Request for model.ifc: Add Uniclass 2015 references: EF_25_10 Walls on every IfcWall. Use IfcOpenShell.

First a look at what the model holds.

```python
import ifcopenshell

model = ifcopenshell.open("model.ifc")
print(model.schema)
print("classifications:", [c.Name for c in model.by_type("IfcClassification")])
for ifc_class in ("IfcDoor", "IfcRoof", "IfcStair", "IfcWall", "IfcWindow"):
    print(ifc_class, len(model.by_type(ifc_class)))
```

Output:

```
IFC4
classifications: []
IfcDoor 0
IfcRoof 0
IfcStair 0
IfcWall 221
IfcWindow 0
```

```python
import ifcopenshell
import ifcopenshell.api.classification

model = ifcopenshell.open("model.ifc")

system = ifcopenshell.api.classification.add_classification(model, classification="Uniclass 2015")

codes = {
    "IfcWall": ("EF_25_10", "Walls"),
}
for ifc_class, (code, name) in codes.items():
    products = model.by_type(ifc_class)
    ifcopenshell.api.classification.add_reference(
        model, products=products, classification=system, identification=code, name=name
    )
    print(code, len(products))

model.write("model_updated.ifc")
```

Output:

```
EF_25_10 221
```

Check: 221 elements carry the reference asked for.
